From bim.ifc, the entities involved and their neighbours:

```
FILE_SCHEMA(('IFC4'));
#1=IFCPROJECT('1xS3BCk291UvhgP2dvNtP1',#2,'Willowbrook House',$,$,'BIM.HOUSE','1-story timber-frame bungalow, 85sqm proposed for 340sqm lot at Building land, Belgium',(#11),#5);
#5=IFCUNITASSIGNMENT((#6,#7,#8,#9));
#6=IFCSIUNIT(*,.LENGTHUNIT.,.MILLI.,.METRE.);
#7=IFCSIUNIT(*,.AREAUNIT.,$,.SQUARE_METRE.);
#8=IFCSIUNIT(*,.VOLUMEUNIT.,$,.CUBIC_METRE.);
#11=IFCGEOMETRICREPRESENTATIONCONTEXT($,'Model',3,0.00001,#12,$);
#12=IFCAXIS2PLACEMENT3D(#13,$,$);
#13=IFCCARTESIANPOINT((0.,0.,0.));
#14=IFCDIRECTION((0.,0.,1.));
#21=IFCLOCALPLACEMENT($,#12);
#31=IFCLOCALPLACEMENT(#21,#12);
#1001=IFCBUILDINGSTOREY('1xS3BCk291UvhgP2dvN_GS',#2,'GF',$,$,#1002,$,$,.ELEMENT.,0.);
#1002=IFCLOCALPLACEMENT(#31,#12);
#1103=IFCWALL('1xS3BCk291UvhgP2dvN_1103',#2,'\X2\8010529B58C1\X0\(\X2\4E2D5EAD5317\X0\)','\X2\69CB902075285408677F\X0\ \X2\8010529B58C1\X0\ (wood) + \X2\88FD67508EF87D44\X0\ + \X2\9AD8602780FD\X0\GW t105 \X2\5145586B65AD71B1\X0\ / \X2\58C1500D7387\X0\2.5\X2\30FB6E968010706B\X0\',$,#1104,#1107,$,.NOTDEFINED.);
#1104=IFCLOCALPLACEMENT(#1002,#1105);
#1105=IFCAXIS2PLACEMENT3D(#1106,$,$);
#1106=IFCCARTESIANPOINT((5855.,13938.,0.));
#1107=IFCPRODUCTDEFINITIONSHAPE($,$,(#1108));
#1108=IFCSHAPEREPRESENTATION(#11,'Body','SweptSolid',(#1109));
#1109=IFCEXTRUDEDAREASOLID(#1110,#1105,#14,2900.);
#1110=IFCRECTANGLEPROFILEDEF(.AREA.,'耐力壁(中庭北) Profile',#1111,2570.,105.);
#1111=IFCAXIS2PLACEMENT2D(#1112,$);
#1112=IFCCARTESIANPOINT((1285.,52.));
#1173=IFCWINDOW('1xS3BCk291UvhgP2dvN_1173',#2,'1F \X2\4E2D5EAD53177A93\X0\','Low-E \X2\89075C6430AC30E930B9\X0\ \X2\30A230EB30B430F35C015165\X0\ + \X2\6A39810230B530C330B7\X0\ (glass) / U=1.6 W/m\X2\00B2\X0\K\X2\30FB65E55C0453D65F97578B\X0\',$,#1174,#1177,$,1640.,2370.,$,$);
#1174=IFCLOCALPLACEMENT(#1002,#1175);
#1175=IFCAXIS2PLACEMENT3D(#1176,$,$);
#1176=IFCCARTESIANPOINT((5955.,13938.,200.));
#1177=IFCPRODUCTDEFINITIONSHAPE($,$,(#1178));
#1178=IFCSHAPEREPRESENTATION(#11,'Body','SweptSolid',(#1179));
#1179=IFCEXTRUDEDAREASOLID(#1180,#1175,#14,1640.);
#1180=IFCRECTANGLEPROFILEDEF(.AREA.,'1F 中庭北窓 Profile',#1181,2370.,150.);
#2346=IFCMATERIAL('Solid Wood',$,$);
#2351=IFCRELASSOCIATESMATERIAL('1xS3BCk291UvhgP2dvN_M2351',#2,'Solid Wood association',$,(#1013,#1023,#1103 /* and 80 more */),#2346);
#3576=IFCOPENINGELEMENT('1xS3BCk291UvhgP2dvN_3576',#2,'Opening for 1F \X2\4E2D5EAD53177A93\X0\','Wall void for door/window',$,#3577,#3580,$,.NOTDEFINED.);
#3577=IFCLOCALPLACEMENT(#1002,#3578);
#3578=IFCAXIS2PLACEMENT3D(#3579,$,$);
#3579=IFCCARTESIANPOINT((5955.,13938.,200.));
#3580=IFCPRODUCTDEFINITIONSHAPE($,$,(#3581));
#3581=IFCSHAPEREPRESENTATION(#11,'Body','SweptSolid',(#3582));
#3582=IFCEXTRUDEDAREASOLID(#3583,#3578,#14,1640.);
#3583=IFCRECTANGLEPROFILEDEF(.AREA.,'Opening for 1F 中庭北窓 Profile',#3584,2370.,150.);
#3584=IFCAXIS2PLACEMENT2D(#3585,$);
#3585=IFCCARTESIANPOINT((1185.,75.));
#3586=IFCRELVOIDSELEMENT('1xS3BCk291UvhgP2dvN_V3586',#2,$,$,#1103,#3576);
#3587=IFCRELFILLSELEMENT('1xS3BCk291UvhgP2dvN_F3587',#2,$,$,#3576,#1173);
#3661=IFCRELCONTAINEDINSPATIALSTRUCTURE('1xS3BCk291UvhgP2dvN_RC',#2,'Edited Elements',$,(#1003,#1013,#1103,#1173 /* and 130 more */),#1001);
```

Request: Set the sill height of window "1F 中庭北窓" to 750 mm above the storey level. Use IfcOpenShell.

```python
import numpy as np
import ifcopenshell
import ifcopenshell.api.geometry
import ifcopenshell.geom
import ifcopenshell.util.element
import ifcopenshell.util.placement
import ifcopenshell.util.shape
import ifcopenshell.util.unit

model = ifcopenshell.open("bim.ifc")
unit_scale = ifcopenshell.util.unit.calculate_unit_scale(model)

window = model.by_guid("1xS3BCk291UvhgP2dvN_1173")
opening = window.FillsVoids[0].RelatingOpeningElement
storey = ifcopenshell.util.element.get_container(window, ifc_class="IfcBuildingStorey")
level = ifcopenshell.util.placement.get_local_placement(storey.ObjectPlacement)[2, 3]

# The opening's origin need not be at the sill, so measure its lowest point.
shape = ifcopenshell.geom.create_shape(ifcopenshell.geom.settings(), opening)
bottom = ifcopenshell.util.shape.get_shape_bottom_elevation(shape, shape.geometry) / unit_scale
dz = level + 0.75 / unit_scale - bottom

shift = np.array([0.0, 0.0, dz])
# The window is not placed relative to its opening, so move both.
for product in (opening, window):
    matrix = ifcopenshell.util.placement.get_local_placement(product.ObjectPlacement)
    matrix[:3, 3] += shift
    ifcopenshell.api.geometry.edit_object_placement(model, product=product, matrix=matrix, is_si=False)

print(f"moved by {dz * unit_scale:+.3f} m")

model.write("bim-out.ifc")
```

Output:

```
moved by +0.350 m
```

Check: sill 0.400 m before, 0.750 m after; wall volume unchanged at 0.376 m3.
